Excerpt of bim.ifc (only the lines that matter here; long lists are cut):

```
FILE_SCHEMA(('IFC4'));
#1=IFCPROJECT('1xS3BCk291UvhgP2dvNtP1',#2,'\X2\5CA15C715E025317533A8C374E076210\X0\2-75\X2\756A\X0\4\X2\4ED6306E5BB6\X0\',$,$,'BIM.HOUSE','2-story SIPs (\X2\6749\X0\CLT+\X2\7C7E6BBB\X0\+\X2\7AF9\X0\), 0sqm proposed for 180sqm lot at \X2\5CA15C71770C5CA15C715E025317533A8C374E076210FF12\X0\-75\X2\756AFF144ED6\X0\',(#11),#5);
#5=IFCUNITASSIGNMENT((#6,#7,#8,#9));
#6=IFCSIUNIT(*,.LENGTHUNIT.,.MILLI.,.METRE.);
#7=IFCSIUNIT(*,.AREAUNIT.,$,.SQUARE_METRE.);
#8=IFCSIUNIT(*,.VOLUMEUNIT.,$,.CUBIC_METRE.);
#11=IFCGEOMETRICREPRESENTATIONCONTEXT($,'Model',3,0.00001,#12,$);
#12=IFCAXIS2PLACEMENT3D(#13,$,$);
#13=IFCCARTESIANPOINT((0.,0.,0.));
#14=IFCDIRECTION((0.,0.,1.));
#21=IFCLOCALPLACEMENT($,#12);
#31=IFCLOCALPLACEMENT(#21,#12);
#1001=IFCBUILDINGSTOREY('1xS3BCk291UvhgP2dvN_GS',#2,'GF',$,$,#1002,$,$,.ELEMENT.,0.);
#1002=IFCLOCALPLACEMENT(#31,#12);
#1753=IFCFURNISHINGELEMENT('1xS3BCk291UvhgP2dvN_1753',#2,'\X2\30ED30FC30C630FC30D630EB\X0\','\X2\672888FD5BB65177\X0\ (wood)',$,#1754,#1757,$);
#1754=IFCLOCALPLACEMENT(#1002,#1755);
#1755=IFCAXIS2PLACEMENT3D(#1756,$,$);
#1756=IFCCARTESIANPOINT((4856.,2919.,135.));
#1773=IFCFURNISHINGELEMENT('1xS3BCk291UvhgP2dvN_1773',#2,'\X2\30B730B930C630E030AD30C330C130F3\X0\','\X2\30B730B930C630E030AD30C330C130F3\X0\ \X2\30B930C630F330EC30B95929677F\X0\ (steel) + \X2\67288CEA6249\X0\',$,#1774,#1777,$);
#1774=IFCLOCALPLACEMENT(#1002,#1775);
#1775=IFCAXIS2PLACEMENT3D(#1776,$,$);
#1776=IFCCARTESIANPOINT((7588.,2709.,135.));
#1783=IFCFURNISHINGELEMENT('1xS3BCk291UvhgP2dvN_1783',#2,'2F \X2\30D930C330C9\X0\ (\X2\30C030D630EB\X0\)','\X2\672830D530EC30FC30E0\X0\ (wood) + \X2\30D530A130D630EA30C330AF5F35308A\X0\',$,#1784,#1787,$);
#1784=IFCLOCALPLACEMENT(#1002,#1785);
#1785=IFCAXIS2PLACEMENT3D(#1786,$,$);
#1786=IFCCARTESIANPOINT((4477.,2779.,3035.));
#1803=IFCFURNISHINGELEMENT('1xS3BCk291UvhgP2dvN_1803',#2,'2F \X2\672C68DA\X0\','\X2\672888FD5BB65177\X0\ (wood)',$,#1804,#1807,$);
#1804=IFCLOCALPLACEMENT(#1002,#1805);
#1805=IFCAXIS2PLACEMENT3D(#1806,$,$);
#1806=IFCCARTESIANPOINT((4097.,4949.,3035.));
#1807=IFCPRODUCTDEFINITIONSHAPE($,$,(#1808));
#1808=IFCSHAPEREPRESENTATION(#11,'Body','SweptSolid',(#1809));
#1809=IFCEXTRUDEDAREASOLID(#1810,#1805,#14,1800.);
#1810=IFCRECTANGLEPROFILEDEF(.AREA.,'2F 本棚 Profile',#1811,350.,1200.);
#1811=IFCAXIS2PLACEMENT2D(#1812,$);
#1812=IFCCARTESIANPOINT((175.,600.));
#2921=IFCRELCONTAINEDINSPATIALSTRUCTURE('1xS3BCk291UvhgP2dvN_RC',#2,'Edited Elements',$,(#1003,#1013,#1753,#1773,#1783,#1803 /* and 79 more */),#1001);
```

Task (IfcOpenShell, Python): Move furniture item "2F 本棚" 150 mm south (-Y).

```python
import ifcopenshell
import ifcopenshell.api.geometry
import ifcopenshell.util.placement
import ifcopenshell.util.unit

model = ifcopenshell.open("bim.ifc")
unit_scale = ifcopenshell.util.unit.calculate_unit_scale(model)

item = model.by_guid("1xS3BCk291UvhgP2dvN_1803")
matrix = ifcopenshell.util.placement.get_local_placement(item.ObjectPlacement)
matrix[1, 3] -= 0.15 / unit_scale
ifcopenshell.api.geometry.edit_object_placement(model, product=item, matrix=matrix, is_si=False)

print(ifcopenshell.util.placement.get_local_placement(item.ObjectPlacement).round(3) + 0.0)

model.write("bim_v2.ifc")
```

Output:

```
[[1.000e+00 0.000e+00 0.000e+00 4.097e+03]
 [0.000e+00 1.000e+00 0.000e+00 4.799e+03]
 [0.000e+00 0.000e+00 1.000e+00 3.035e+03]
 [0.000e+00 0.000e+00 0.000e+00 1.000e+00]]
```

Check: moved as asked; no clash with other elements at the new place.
